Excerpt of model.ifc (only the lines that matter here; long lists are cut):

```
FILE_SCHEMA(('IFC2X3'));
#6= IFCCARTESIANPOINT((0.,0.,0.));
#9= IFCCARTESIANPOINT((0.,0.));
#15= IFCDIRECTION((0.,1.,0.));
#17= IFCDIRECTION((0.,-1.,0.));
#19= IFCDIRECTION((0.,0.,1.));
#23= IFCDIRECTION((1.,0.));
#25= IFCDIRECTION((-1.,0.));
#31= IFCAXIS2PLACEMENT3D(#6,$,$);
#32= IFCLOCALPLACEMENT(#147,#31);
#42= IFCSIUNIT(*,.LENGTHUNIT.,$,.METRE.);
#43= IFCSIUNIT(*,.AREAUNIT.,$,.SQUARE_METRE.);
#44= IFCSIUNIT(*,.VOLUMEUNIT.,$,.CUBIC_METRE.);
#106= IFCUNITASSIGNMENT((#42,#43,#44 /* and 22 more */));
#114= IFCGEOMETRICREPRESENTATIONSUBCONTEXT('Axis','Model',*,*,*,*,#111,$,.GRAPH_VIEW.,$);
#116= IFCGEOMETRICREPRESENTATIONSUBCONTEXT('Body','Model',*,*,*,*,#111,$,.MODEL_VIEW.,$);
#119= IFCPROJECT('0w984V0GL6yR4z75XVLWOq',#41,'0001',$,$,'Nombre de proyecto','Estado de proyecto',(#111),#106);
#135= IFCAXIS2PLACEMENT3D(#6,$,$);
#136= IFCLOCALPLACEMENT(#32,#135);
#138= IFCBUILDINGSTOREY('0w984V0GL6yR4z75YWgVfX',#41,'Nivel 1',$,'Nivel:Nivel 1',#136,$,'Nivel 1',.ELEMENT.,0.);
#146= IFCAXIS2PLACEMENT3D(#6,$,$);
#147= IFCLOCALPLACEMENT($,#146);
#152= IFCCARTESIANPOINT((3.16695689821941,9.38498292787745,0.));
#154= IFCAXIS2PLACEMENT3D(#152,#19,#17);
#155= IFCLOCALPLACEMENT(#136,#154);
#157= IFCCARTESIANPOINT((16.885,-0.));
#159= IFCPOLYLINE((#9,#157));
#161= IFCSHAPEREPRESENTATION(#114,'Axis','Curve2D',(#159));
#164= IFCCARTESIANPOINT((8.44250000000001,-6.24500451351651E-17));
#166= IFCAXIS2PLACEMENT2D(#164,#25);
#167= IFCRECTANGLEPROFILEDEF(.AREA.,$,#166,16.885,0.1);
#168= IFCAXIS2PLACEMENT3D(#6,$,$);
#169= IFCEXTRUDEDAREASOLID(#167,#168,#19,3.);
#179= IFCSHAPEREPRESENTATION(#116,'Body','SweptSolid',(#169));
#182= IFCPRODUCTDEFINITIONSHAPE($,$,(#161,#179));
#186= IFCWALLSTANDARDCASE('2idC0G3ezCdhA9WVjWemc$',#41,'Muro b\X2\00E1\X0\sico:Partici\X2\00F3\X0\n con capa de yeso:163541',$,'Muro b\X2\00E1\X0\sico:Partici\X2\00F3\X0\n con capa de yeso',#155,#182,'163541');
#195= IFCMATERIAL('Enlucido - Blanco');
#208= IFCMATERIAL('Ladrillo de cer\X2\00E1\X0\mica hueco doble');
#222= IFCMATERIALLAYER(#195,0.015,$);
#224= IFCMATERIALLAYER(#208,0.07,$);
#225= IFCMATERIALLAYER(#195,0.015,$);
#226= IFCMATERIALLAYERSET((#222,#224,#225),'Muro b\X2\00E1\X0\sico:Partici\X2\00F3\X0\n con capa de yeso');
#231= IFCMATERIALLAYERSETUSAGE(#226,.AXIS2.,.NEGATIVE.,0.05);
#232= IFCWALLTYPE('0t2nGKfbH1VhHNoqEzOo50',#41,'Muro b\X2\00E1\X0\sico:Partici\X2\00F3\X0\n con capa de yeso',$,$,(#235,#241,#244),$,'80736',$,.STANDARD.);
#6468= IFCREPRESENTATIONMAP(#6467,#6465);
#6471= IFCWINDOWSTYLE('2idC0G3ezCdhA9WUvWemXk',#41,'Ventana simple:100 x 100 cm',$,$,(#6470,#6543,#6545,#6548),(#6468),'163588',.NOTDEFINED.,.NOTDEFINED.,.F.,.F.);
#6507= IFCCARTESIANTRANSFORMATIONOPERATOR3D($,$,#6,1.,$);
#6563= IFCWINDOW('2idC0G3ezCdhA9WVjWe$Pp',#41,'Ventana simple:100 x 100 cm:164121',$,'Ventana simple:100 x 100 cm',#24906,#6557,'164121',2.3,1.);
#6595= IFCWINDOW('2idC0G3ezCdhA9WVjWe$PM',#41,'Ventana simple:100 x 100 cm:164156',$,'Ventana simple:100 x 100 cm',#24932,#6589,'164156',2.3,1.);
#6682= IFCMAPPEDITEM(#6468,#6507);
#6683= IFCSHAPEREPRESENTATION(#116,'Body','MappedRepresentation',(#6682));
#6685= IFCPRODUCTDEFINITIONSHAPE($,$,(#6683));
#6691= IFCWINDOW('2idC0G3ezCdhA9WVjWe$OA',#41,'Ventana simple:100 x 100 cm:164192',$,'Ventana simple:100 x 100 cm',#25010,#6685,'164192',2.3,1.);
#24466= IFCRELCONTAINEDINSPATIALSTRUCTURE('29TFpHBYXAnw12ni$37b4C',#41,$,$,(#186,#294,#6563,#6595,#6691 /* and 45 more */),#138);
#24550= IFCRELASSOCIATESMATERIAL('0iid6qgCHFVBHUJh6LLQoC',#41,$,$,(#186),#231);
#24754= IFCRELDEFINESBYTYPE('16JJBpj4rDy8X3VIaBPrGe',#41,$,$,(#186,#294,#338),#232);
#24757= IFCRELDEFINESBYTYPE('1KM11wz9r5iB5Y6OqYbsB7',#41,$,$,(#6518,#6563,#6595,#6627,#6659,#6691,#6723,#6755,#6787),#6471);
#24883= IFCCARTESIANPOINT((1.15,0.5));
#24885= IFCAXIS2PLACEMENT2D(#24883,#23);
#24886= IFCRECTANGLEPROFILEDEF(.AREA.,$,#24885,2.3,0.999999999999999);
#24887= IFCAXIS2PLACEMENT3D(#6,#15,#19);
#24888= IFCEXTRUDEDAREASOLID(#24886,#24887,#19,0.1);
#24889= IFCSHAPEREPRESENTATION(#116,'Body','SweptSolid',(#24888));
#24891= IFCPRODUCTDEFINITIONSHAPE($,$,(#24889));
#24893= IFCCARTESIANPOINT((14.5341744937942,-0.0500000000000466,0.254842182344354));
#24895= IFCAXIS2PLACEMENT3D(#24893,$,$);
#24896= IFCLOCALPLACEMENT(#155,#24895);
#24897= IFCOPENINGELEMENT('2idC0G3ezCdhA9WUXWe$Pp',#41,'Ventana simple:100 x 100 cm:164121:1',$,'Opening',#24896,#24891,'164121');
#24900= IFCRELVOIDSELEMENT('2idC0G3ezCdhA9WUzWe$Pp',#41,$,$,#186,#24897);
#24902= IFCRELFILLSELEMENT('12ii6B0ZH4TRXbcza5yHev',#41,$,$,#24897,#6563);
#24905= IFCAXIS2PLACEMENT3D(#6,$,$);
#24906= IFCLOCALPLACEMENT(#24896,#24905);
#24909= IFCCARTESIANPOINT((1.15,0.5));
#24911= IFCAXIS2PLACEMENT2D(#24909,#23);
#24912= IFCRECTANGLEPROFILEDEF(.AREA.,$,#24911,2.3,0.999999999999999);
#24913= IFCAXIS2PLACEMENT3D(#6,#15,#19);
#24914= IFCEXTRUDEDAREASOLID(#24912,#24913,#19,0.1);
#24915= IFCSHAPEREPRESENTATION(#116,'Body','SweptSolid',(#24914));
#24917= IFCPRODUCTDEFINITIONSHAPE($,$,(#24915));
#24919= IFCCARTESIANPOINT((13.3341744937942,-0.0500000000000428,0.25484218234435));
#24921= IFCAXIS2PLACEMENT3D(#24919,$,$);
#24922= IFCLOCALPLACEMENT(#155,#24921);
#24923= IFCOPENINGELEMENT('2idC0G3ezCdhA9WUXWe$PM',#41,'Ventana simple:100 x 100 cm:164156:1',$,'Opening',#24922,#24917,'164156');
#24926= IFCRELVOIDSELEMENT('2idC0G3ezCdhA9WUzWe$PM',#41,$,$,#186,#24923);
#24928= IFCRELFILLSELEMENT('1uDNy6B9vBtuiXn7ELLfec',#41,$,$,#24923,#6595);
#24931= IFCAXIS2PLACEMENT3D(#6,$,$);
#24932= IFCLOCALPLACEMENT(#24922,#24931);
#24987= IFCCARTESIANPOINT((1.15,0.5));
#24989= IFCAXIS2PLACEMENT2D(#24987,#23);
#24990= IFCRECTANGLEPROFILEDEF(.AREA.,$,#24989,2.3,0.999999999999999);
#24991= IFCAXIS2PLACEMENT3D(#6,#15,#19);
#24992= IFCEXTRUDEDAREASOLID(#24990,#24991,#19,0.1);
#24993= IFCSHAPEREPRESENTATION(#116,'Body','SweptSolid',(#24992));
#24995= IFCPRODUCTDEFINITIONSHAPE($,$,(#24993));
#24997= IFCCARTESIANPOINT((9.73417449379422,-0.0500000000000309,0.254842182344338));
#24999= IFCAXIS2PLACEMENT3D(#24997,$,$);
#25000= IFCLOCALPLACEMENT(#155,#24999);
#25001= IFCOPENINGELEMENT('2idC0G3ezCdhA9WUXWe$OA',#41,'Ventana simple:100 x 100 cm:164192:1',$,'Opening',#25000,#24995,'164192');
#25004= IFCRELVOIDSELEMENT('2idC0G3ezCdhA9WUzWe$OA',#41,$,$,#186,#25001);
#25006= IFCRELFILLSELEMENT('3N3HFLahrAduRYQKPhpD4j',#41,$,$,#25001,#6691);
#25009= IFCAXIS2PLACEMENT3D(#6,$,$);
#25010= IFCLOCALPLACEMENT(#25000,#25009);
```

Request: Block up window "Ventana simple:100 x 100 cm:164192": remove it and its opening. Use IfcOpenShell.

```python
import ifcopenshell
import ifcopenshell.api.feature
import ifcopenshell.api.root
import ifcopenshell.geom
import ifcopenshell.util.shape

model = ifcopenshell.open("model.ifc")
settings = ifcopenshell.geom.settings()


def volume(element):
    """Net volume in cubic metres, openings subtracted."""
    shape = ifcopenshell.geom.create_shape(settings, element)
    return ifcopenshell.util.shape.get_volume(shape.geometry)


window = model.by_guid("2idC0G3ezCdhA9WVjWe$OA")
opening = window.FillsVoids[0].RelatingOpeningElement
wall = opening.VoidsElements[0].RelatingBuildingElement
before = volume(wall)

ifcopenshell.api.root.remove_product(model, product=window)
ifcopenshell.api.feature.remove_feature(model, feature=opening)

after = volume(wall)

print(f"wall volume {before:.3f} -> {after:.3f} m3")

model.write("model_v2.ifc")
```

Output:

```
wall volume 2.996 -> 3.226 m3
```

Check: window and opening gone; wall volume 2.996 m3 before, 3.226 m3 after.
